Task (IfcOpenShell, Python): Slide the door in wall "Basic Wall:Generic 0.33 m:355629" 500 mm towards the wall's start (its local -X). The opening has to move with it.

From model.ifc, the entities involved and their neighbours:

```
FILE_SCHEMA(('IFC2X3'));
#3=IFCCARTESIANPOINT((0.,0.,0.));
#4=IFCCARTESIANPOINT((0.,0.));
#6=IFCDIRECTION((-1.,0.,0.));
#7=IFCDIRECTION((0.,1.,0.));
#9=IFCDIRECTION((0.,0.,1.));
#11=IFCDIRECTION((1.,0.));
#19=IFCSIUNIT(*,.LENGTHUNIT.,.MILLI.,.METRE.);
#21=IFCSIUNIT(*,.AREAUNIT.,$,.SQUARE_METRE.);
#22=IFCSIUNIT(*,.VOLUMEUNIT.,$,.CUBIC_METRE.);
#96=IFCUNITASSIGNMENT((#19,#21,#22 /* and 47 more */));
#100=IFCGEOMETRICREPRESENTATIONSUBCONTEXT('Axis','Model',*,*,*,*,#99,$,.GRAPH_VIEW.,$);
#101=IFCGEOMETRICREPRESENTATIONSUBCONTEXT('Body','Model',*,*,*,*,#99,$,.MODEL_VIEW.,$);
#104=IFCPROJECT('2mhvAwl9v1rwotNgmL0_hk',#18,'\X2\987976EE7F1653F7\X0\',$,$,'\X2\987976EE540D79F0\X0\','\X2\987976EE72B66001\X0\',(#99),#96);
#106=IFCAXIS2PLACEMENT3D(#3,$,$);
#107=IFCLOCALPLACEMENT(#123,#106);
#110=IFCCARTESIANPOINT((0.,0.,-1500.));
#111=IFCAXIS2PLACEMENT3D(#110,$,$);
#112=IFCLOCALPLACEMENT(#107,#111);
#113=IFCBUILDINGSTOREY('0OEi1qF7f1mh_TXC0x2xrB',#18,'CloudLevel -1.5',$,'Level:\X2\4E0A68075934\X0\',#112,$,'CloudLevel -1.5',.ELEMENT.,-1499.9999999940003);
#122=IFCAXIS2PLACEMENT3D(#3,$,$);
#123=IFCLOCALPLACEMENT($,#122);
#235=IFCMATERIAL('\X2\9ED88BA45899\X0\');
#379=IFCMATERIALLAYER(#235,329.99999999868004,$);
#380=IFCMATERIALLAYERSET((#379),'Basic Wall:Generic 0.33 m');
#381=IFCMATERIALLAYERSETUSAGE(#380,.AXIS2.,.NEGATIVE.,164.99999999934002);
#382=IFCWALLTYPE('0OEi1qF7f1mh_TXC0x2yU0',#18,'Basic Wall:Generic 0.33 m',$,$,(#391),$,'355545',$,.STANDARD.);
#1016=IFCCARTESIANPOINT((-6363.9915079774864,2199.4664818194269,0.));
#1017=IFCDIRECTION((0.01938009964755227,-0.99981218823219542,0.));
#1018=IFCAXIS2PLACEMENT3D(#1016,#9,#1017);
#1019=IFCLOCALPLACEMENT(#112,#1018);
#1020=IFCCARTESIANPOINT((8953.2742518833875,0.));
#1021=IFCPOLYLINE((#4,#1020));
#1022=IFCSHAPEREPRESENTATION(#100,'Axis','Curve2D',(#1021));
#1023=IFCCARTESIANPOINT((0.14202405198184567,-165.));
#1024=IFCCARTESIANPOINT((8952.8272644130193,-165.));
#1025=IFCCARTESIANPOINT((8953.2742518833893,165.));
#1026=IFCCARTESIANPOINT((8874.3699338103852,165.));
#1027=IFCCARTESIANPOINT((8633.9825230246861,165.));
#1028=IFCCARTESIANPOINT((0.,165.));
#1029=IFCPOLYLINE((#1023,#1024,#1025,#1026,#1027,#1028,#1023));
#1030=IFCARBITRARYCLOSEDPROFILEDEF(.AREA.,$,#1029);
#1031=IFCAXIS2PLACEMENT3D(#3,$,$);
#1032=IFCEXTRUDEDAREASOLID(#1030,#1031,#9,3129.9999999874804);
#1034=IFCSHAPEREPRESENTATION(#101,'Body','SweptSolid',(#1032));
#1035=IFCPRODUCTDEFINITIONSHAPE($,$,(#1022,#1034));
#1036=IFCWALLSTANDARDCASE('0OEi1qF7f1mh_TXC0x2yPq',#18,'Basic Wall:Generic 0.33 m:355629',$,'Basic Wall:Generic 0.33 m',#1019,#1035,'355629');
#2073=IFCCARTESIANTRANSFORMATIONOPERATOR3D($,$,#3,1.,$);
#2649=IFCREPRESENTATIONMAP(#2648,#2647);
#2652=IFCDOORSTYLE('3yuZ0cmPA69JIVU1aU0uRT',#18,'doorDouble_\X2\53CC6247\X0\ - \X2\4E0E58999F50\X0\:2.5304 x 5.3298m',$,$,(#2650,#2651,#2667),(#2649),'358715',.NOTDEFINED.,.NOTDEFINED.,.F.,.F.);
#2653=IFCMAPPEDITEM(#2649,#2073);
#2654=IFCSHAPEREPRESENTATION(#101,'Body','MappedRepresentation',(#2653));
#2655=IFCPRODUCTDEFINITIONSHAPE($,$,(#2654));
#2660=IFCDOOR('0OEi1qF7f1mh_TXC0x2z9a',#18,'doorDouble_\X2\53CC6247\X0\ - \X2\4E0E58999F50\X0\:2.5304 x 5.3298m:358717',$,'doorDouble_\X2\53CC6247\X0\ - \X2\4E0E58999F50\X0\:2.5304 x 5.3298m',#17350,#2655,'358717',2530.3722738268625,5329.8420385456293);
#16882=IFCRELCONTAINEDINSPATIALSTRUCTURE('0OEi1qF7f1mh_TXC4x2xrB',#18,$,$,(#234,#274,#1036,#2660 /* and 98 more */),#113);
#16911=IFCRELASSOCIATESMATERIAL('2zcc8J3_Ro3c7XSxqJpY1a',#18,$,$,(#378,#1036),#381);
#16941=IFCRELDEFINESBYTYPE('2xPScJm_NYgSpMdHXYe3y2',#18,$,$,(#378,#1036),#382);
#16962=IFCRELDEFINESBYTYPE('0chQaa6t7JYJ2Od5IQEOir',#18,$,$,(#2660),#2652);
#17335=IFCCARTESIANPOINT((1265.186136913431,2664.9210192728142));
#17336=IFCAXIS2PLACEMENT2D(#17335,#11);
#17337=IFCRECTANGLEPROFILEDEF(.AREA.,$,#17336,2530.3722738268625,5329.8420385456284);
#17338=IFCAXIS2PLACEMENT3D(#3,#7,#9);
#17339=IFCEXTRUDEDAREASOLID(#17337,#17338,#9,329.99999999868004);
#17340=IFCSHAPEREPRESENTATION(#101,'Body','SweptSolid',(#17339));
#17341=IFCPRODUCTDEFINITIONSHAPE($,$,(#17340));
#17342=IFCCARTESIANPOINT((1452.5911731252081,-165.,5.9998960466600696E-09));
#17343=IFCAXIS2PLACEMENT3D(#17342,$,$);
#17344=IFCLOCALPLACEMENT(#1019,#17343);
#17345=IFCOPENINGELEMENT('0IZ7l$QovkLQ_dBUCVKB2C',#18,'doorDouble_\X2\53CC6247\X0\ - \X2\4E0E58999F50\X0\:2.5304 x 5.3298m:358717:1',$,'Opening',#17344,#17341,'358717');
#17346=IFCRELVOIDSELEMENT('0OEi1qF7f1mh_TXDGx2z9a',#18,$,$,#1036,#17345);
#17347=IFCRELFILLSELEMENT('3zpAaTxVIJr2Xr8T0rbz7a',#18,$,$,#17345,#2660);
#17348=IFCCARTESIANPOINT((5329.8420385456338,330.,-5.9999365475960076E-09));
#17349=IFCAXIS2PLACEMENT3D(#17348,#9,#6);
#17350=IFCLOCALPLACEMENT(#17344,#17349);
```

```python
import ifcopenshell
import ifcopenshell.api.geometry
import ifcopenshell.util.placement

model = ifcopenshell.open("model.ifc")

door = model.by_guid("0OEi1qF7f1mh_TXC0x2z9a")
opening = door.FillsVoids[0].RelatingOpeningElement
wall = opening.VoidsElements[0].RelatingBuildingElement

wall_matrix = ifcopenshell.util.placement.get_local_placement(wall.ObjectPlacement)
shift = wall_matrix[:3, 0] * -500.0
before = ifcopenshell.util.placement.get_local_placement(door.ObjectPlacement)[:3, 3].copy()

# The door is placed relative to its opening, so it follows when the opening moves.
matrix = ifcopenshell.util.placement.get_local_placement(opening.ObjectPlacement)
matrix[:3, 3] += shift
ifcopenshell.api.geometry.edit_object_placement(
    model, product=opening, matrix=matrix, is_si=False, should_transform_children=True
)

after = ifcopenshell.util.placement.get_local_placement(door.ObjectPlacement)[:3, 3]
print("door moved by", (after - before).round(3) + 0.0)

model.write("model-out.ifc")
```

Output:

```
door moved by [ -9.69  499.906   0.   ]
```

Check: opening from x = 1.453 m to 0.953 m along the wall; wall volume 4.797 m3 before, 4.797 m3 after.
